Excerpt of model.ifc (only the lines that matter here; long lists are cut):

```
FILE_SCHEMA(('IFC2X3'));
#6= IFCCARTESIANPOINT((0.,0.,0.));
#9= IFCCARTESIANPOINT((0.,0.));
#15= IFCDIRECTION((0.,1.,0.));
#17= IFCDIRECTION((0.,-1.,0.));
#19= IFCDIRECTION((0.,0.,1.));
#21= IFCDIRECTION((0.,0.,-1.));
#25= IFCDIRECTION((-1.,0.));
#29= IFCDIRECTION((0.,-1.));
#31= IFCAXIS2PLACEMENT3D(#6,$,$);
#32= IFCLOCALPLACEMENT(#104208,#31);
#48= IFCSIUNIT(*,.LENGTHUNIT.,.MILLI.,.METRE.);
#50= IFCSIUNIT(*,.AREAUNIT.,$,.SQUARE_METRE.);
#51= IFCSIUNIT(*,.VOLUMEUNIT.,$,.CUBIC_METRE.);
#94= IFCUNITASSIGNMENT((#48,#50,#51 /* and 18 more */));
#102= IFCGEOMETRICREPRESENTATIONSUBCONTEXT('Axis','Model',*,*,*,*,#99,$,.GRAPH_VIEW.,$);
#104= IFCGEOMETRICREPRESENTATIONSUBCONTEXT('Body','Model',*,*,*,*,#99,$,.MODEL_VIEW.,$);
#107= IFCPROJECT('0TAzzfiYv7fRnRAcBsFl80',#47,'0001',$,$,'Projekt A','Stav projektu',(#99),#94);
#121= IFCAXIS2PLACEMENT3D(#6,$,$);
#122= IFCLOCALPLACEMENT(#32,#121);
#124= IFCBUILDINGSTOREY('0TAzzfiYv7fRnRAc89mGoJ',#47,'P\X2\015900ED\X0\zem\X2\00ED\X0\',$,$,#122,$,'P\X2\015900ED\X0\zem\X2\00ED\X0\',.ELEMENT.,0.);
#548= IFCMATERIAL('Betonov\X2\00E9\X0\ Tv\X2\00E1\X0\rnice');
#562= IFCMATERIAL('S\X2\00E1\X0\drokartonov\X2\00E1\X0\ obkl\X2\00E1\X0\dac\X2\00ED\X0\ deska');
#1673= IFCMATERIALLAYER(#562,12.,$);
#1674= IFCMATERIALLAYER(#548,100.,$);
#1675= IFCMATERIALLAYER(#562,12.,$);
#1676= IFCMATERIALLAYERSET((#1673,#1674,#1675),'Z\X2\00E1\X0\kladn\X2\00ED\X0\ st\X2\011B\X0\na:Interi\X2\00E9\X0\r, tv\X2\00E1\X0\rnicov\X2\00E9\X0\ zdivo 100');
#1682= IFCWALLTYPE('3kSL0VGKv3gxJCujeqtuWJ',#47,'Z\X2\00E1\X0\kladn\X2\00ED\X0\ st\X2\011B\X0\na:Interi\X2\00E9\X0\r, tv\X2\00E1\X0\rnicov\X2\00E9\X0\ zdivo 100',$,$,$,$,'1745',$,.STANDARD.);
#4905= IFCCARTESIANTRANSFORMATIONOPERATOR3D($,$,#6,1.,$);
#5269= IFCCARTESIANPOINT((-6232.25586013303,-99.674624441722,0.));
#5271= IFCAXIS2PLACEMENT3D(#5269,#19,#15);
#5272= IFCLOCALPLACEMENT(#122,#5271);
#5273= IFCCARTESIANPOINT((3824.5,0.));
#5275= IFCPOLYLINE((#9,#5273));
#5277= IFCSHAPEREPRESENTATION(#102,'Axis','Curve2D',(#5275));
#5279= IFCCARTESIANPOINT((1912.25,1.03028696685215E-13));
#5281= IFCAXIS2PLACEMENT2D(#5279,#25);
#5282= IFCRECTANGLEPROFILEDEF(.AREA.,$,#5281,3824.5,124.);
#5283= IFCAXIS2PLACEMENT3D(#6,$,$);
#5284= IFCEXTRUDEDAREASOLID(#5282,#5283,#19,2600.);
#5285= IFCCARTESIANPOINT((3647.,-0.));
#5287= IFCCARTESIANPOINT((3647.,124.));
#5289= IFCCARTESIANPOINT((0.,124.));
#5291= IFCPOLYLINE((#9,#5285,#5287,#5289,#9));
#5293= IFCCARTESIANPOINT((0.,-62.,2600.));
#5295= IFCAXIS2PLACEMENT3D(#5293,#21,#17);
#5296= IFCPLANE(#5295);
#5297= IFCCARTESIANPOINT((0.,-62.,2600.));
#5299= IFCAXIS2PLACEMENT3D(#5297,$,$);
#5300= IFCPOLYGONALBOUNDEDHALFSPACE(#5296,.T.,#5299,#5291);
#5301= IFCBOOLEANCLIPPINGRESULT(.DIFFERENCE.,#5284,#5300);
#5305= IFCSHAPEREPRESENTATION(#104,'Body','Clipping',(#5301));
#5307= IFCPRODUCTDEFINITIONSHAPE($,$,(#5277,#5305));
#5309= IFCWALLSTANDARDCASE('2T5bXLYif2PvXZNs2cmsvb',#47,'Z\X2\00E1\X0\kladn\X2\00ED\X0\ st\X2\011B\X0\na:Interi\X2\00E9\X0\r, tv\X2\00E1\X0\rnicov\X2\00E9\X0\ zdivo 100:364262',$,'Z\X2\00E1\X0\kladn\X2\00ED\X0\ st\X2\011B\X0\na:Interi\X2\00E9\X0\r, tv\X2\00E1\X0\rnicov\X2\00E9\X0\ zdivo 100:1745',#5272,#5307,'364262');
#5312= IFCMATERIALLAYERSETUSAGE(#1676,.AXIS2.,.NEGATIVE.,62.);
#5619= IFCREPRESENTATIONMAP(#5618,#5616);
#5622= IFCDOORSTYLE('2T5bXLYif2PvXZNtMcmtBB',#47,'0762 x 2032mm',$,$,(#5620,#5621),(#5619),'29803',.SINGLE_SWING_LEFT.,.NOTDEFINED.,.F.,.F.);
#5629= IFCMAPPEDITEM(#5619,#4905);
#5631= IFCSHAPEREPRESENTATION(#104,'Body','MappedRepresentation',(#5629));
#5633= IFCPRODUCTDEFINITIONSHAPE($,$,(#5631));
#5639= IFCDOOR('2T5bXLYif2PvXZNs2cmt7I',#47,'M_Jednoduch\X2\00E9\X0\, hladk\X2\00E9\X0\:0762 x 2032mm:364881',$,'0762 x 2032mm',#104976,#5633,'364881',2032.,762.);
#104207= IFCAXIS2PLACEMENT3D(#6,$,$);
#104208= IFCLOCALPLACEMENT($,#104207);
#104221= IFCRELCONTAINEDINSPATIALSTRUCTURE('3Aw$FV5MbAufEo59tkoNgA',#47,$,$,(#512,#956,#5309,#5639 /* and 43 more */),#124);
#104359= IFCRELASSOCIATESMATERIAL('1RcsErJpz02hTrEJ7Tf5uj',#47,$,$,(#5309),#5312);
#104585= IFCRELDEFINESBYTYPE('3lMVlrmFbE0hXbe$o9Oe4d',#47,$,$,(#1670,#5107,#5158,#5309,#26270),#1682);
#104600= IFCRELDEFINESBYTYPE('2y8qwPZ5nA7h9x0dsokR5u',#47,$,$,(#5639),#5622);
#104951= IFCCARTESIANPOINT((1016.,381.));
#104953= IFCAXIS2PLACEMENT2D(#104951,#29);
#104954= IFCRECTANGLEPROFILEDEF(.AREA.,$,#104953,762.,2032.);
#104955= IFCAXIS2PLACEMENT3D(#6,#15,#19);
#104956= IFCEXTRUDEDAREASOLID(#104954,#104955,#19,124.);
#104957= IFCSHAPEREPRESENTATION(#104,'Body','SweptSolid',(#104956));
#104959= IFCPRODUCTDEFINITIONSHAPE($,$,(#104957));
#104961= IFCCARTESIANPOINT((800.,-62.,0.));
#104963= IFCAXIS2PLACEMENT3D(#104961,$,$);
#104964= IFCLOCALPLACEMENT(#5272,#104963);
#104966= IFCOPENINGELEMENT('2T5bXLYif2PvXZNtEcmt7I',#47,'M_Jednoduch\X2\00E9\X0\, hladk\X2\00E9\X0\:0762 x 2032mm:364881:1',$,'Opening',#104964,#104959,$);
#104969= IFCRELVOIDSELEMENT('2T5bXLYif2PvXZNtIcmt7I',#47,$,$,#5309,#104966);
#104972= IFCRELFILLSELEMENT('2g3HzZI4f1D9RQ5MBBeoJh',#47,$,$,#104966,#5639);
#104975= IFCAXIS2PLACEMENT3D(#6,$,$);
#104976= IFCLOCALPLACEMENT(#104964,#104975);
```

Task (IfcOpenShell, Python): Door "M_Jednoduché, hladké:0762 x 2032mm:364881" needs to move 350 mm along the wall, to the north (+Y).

```python
import ifcopenshell
import ifcopenshell.api.geometry
import ifcopenshell.util.placement
import ifcopenshell.util.unit

model = ifcopenshell.open("model.ifc")
unit_scale = ifcopenshell.util.unit.calculate_unit_scale(model)

door = model.by_id(5639)
opening = door.FillsVoids[0].RelatingOpeningElement
wall = opening.VoidsElements[0].RelatingBuildingElement

wall_matrix = ifcopenshell.util.placement.get_local_placement(wall.ObjectPlacement)
shift = wall_matrix[:3, 0] * 0.35 / unit_scale
before = ifcopenshell.util.placement.get_local_placement(door.ObjectPlacement)[:3, 3].copy()

# The door is placed relative to its opening, so it follows when the opening moves.
matrix = ifcopenshell.util.placement.get_local_placement(opening.ObjectPlacement)
matrix[:3, 3] += shift
ifcopenshell.api.geometry.edit_object_placement(
    model, product=opening, matrix=matrix, is_si=False, should_transform_children=True
)

after = ifcopenshell.util.placement.get_local_placement(door.ObjectPlacement)[:3, 3]
print("door moved by", (after - before).round(3) + 0.0)

model.write("model-out.ifc")
```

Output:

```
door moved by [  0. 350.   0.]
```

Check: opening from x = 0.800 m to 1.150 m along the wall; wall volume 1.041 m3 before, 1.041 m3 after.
